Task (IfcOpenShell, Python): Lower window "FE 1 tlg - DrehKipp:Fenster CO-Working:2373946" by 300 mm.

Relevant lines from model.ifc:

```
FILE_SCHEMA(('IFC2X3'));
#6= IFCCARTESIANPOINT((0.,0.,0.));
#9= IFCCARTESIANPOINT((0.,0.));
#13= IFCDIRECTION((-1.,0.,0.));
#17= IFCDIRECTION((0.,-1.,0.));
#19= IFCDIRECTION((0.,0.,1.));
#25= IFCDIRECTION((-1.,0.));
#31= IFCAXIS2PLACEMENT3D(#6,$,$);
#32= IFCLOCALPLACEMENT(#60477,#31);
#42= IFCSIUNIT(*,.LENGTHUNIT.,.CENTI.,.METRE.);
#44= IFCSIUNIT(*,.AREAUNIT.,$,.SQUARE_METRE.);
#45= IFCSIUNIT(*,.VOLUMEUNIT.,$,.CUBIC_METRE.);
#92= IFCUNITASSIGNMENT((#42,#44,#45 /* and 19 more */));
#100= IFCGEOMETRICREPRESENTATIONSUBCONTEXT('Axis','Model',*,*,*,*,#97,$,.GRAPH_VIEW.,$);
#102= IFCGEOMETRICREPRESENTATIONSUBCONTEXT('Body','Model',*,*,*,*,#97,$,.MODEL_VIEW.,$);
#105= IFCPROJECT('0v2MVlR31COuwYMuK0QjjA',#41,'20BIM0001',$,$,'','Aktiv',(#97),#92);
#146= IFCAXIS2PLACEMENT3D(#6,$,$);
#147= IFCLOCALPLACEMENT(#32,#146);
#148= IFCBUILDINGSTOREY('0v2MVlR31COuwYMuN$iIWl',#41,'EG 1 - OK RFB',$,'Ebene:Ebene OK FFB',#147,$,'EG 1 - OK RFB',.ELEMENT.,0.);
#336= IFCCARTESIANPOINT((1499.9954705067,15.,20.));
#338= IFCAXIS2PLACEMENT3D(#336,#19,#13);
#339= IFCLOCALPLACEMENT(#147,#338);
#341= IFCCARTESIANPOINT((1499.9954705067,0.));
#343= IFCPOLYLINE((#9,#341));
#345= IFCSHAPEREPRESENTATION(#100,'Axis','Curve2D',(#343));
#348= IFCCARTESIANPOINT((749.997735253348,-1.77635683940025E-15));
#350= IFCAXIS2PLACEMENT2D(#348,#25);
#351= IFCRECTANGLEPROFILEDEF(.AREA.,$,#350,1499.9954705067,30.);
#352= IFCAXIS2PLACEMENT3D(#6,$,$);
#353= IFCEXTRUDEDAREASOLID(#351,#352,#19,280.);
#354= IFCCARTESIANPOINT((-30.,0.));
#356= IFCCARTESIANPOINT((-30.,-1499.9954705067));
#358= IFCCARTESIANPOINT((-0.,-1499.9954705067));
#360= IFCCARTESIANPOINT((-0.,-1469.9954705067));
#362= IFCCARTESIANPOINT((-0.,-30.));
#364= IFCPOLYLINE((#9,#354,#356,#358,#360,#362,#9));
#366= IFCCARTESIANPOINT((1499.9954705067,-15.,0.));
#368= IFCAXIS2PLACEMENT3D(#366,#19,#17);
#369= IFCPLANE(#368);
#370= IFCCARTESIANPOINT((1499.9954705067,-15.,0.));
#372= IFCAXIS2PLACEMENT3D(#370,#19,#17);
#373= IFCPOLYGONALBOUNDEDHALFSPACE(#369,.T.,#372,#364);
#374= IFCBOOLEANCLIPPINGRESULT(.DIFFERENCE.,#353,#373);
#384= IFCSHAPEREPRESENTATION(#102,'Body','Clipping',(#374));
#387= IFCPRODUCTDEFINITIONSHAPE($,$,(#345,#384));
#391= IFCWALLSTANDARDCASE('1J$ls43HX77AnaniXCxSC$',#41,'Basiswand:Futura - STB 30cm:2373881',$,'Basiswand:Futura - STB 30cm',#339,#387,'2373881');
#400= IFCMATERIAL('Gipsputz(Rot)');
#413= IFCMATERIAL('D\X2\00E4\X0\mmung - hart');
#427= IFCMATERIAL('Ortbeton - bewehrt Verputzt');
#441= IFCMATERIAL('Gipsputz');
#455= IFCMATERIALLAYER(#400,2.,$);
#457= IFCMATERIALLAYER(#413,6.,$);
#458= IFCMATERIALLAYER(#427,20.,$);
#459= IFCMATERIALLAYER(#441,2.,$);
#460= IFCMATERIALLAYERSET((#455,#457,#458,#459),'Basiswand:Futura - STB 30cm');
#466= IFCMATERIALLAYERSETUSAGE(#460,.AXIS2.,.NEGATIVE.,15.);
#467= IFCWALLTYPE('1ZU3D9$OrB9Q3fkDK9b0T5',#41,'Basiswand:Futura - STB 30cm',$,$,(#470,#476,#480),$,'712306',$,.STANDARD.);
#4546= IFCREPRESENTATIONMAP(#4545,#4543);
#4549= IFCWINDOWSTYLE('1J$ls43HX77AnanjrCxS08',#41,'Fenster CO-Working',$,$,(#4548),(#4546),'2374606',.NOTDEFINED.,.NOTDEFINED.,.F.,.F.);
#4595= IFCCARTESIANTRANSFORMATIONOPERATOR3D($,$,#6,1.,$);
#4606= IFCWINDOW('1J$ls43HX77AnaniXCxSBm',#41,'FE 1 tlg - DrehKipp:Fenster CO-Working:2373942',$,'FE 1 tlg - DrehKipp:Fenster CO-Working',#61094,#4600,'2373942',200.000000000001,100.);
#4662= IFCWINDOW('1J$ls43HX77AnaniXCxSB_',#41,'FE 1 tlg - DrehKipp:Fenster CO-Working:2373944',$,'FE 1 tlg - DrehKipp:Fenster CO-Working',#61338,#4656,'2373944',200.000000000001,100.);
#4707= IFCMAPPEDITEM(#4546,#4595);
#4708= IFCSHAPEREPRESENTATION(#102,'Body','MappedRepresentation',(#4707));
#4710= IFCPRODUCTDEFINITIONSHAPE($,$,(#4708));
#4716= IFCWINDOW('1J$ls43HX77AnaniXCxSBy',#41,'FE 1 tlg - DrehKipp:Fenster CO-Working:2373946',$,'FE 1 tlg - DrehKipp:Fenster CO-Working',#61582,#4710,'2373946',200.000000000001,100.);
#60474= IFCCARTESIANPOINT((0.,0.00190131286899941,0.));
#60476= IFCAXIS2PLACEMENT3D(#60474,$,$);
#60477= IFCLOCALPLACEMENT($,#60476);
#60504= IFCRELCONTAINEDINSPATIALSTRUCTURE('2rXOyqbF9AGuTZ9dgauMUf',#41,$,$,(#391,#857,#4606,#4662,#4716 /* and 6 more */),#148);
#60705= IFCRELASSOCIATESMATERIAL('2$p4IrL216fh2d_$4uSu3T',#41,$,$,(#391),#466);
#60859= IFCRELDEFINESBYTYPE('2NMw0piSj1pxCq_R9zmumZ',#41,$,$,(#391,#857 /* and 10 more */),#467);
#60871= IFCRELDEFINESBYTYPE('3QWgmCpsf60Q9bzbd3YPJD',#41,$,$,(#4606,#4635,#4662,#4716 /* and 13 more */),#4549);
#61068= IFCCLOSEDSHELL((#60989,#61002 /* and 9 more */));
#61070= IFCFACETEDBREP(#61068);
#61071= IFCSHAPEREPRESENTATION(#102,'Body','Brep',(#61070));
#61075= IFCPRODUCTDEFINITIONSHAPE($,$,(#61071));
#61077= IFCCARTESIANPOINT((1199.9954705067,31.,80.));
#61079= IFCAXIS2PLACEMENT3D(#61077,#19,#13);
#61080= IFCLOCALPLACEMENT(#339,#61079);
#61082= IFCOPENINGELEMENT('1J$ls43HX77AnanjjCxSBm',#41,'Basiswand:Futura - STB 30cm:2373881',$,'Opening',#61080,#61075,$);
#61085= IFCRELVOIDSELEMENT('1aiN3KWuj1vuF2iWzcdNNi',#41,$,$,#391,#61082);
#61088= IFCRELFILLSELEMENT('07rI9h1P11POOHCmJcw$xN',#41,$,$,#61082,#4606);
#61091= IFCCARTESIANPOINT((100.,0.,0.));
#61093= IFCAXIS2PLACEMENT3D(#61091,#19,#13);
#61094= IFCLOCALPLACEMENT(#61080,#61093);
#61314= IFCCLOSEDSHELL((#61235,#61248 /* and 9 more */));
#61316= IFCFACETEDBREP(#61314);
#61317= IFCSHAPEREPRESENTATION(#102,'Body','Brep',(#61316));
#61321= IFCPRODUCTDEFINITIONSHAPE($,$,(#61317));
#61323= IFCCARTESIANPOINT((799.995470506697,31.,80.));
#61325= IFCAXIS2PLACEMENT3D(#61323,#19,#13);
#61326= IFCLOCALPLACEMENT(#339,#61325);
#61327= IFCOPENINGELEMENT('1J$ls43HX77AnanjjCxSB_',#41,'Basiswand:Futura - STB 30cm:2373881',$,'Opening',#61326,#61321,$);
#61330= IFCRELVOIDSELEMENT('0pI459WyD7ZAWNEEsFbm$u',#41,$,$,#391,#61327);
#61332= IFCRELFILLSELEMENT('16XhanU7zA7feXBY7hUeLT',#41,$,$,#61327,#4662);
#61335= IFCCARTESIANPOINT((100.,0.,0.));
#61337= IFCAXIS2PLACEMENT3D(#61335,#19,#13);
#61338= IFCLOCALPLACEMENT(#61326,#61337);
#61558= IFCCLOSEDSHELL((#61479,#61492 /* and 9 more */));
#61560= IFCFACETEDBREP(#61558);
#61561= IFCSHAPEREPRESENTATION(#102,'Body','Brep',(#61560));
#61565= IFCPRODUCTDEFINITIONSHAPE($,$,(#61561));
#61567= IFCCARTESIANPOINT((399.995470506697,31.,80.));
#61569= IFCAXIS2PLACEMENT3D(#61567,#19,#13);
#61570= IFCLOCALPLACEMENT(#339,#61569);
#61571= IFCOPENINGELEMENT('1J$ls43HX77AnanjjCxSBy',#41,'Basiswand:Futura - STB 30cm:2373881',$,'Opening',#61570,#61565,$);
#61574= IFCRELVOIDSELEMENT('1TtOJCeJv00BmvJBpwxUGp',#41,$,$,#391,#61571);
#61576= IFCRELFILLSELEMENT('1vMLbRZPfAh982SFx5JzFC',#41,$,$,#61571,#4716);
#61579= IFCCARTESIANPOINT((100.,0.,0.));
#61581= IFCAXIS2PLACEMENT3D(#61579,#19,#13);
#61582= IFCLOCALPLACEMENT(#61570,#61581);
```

```python
import numpy as np
import ifcopenshell
import ifcopenshell.api.geometry
import ifcopenshell.util.placement
import ifcopenshell.util.unit

model = ifcopenshell.open("model.ifc")
unit_scale = ifcopenshell.util.unit.calculate_unit_scale(model)

window = model.by_guid("1J$ls43HX77AnaniXCxSBy")
opening = window.FillsVoids[0].RelatingOpeningElement
dz = -0.3 / unit_scale

shift = np.array([0.0, 0.0, dz])
# The window is placed relative to its opening, so it follows when the opening moves.
matrix = ifcopenshell.util.placement.get_local_placement(opening.ObjectPlacement)
matrix[:3, 3] += shift
ifcopenshell.api.geometry.edit_object_placement(
    model, product=opening, matrix=matrix, is_si=False, should_transform_children=True
)

print(f"moved by {dz * unit_scale:+.3f} m")

model.write("model_v2.ifc")
```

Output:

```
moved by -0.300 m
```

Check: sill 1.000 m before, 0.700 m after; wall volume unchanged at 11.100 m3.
